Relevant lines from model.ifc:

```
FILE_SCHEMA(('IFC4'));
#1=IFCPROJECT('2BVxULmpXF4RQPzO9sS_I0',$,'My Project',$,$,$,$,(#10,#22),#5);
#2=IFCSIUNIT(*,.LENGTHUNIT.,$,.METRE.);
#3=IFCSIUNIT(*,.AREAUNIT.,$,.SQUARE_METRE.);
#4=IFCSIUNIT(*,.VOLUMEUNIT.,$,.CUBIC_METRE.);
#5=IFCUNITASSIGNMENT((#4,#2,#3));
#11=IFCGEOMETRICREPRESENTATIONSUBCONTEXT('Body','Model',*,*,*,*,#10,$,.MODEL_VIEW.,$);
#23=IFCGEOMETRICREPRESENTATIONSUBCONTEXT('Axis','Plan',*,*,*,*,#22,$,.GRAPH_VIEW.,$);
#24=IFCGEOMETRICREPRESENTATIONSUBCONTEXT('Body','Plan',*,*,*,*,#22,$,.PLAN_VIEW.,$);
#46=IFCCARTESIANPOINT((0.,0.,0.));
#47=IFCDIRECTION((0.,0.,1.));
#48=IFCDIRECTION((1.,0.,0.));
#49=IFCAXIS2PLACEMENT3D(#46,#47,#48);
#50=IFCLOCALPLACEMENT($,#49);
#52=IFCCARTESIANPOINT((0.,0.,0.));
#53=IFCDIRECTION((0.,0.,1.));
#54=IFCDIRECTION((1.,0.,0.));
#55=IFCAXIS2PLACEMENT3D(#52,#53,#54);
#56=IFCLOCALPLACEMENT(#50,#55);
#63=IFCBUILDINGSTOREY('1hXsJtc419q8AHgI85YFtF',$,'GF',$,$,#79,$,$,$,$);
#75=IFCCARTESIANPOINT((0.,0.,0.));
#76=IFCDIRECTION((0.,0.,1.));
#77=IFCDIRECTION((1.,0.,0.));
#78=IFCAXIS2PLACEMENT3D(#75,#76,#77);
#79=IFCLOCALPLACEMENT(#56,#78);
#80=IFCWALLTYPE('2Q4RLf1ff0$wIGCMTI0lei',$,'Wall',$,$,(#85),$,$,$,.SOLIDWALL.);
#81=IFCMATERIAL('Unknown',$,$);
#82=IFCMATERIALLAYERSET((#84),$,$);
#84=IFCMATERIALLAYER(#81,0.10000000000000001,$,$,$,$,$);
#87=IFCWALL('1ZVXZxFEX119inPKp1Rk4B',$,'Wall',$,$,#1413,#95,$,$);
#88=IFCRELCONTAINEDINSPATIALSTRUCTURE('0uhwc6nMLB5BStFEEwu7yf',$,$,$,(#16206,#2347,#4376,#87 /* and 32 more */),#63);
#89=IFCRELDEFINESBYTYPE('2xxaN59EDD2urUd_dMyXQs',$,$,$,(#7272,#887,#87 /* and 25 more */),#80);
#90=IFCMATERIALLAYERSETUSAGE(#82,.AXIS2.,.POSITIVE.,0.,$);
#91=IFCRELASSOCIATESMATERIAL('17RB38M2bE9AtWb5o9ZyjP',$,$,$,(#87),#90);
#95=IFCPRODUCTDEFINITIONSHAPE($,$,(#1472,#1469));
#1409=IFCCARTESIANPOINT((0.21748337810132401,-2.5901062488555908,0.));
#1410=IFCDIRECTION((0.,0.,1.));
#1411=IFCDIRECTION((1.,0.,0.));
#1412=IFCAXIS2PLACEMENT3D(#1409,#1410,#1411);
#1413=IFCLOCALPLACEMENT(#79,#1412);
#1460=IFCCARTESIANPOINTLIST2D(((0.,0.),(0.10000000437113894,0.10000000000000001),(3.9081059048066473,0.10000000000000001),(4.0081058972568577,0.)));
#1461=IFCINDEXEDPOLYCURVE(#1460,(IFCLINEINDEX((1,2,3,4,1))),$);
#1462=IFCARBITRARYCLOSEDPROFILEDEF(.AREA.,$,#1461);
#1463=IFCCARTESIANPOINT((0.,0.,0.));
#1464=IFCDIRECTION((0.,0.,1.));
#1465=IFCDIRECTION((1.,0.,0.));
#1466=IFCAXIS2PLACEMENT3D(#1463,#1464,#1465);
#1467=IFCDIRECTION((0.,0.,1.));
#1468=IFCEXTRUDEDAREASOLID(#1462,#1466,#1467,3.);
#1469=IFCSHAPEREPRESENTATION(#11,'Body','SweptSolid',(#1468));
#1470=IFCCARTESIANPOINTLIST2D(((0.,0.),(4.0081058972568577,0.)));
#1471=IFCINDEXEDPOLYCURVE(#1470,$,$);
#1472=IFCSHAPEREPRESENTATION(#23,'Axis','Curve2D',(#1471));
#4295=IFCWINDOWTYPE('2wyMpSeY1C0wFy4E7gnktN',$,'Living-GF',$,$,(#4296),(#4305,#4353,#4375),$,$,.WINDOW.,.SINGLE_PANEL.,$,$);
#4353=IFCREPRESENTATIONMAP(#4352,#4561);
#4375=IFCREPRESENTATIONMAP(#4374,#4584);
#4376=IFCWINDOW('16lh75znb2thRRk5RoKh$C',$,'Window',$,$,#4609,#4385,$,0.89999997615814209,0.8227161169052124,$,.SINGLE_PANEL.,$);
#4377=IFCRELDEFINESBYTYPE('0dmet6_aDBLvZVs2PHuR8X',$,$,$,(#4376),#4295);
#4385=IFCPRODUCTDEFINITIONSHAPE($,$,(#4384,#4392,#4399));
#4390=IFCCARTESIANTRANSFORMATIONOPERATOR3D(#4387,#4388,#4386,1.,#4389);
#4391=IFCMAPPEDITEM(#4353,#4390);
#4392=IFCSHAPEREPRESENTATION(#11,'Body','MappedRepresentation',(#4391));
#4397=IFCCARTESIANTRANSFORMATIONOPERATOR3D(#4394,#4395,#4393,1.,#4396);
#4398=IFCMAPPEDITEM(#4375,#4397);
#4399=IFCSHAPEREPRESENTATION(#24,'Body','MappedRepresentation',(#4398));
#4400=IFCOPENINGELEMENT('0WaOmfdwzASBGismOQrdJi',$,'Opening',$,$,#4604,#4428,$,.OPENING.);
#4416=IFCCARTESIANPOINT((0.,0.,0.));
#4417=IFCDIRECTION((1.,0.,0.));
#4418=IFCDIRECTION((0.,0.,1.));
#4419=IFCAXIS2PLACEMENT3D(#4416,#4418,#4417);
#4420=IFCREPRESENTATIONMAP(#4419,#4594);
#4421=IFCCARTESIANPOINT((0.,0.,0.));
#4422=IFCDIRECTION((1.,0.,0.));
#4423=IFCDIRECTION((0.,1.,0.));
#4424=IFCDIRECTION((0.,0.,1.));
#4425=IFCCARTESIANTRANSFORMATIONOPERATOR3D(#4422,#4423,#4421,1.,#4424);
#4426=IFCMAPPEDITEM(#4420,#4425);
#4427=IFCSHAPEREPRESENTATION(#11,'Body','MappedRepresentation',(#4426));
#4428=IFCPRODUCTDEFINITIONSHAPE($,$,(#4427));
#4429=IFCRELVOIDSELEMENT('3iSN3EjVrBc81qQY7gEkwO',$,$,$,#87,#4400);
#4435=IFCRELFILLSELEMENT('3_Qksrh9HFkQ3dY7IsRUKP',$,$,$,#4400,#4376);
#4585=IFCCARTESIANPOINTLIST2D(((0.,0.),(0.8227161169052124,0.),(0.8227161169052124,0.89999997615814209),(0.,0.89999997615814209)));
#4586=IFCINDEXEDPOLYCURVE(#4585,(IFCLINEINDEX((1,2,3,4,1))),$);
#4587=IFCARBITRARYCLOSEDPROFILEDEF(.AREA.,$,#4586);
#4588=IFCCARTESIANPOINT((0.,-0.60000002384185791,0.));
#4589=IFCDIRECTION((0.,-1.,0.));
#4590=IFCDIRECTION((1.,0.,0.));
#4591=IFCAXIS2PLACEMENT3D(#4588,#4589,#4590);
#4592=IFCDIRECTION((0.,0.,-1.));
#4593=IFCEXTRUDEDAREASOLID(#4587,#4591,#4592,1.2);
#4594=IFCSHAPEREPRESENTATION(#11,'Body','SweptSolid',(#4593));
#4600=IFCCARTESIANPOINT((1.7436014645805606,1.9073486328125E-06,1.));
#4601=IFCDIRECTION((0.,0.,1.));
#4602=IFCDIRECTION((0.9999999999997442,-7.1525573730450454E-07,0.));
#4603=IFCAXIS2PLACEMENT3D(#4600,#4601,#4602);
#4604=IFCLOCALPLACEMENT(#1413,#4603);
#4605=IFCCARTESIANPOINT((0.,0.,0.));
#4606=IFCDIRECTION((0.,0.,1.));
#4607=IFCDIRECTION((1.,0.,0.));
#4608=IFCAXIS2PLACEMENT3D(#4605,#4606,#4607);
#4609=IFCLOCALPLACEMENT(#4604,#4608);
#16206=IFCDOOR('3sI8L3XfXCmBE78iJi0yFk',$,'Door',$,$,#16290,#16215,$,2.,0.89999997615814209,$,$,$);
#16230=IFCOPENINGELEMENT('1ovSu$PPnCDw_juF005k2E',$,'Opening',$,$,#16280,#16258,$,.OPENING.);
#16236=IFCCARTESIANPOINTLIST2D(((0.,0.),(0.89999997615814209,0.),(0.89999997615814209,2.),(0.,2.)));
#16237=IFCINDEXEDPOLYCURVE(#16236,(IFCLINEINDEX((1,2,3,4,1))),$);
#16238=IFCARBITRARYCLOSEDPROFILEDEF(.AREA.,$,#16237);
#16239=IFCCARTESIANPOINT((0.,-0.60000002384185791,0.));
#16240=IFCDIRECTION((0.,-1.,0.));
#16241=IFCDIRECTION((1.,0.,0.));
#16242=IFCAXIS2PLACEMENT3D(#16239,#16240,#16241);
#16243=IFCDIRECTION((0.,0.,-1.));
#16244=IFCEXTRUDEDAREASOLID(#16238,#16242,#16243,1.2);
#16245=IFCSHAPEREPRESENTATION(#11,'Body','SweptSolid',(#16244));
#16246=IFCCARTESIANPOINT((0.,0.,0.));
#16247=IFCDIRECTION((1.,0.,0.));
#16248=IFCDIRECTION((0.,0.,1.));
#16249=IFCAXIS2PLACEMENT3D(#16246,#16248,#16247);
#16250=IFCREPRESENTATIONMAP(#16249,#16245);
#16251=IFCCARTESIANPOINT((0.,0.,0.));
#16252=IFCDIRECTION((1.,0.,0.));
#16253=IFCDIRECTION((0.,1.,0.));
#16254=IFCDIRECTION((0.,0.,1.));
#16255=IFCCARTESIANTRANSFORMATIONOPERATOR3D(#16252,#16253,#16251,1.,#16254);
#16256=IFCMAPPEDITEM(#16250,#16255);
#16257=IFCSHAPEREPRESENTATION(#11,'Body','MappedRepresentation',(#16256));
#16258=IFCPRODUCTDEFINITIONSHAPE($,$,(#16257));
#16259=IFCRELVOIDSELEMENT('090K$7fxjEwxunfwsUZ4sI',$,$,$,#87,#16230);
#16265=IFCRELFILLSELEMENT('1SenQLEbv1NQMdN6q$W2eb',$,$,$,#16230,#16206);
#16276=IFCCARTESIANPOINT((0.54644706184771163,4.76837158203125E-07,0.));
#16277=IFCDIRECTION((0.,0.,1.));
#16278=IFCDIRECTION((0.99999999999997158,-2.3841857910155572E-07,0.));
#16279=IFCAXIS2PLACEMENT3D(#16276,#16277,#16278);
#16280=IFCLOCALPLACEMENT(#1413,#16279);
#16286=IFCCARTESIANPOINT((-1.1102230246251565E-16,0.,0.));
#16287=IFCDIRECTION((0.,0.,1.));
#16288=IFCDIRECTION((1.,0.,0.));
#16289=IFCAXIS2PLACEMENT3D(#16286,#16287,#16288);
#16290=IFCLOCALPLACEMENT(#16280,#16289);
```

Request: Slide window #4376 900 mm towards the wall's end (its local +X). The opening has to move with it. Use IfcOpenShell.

```python
import ifcopenshell
import ifcopenshell.api.geometry
import ifcopenshell.util.placement
import ifcopenshell.util.unit

model = ifcopenshell.open("model.ifc")
unit_scale = ifcopenshell.util.unit.calculate_unit_scale(model)

window = model.by_id(4376)
opening = window.FillsVoids[0].RelatingOpeningElement
wall = opening.VoidsElements[0].RelatingBuildingElement

wall_matrix = ifcopenshell.util.placement.get_local_placement(wall.ObjectPlacement)
shift = wall_matrix[:3, 0] * 0.9 / unit_scale
before = ifcopenshell.util.placement.get_local_placement(window.ObjectPlacement)[:3, 3].copy()

# The window is placed relative to its opening, so it follows when the opening moves.
matrix = ifcopenshell.util.placement.get_local_placement(opening.ObjectPlacement)
matrix[:3, 3] += shift
ifcopenshell.api.geometry.edit_object_placement(
    model, product=opening, matrix=matrix, is_si=False, should_transform_children=True
)

after = ifcopenshell.util.placement.get_local_placement(window.ObjectPlacement)[:3, 3]
print("window moved by", (after - before).round(3) + 0.0)

model.write("model-out.ifc")
```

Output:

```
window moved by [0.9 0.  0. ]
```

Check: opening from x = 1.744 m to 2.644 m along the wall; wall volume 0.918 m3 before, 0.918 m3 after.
